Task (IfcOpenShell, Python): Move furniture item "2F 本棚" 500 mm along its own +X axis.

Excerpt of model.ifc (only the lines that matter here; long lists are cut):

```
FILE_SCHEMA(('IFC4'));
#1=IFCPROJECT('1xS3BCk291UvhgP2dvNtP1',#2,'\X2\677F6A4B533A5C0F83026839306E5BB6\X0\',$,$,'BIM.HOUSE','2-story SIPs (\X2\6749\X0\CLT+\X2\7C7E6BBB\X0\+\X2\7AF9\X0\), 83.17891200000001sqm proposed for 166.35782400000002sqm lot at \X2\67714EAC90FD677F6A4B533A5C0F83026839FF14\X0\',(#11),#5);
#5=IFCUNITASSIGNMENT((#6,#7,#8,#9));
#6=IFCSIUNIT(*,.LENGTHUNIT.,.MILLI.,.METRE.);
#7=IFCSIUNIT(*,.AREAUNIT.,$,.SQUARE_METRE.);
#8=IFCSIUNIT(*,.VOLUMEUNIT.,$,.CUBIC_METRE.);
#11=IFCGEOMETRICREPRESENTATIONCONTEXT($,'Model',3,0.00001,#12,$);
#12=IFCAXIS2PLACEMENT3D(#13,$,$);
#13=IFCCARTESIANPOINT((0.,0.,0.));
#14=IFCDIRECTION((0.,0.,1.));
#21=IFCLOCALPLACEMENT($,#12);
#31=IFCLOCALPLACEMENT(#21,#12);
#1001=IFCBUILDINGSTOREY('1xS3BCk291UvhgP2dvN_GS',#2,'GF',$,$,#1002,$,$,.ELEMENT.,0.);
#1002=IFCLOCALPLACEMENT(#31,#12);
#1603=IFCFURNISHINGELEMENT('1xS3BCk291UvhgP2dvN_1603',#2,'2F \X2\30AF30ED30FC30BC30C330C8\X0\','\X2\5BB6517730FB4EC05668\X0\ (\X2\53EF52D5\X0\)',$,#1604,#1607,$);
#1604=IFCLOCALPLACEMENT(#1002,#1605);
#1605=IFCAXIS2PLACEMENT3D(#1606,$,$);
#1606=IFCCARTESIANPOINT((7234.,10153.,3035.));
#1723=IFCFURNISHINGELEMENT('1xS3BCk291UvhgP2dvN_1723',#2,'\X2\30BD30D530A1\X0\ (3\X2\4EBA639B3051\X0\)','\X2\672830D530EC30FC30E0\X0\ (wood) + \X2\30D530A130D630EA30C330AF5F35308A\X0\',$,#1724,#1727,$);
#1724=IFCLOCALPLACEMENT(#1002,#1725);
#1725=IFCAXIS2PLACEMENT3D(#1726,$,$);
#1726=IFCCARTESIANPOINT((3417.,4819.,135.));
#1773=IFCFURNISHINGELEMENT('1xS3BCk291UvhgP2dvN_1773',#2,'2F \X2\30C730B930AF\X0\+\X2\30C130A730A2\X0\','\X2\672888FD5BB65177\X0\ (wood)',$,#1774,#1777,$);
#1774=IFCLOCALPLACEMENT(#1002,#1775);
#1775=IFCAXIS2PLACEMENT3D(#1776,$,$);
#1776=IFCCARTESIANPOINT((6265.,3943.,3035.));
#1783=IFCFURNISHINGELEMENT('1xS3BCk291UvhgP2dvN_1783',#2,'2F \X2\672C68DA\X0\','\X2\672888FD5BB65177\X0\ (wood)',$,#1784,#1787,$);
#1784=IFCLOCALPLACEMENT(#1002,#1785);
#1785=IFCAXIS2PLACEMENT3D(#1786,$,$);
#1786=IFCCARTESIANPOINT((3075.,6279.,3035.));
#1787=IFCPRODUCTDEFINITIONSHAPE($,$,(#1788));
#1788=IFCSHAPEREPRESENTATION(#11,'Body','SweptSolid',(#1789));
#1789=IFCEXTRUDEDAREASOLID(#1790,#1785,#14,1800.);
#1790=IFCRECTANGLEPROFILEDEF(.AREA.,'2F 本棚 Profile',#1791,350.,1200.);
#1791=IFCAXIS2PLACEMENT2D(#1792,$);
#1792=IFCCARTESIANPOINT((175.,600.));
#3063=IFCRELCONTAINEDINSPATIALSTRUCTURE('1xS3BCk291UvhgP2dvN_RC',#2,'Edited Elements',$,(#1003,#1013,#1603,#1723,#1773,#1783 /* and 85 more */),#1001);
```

```python
import ifcopenshell
import ifcopenshell.api.geometry
import ifcopenshell.util.placement

model = ifcopenshell.open("model.ifc")

item = model.by_guid("1xS3BCk291UvhgP2dvN_1783")
matrix = ifcopenshell.util.placement.get_local_placement(item.ObjectPlacement)
matrix[:3, 3] += matrix[:3, 0] * 500.0
ifcopenshell.api.geometry.edit_object_placement(model, product=item, matrix=matrix, is_si=False)

print(ifcopenshell.util.placement.get_local_placement(item.ObjectPlacement).round(3) + 0.0)

model.write("model_updated.ifc")
```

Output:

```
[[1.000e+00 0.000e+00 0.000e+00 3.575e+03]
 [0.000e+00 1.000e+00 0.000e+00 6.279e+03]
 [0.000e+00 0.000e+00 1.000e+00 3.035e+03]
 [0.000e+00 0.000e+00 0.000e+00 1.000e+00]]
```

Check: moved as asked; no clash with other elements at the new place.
